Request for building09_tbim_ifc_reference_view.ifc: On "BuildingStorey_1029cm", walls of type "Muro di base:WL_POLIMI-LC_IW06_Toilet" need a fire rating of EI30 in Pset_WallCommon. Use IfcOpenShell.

First a look at what the model holds.

```python
import ifcopenshell
import ifcopenshell.util.element

model = ifcopenshell.open("building09_tbim_ifc_reference_view.ifc")
print(model.schema)
storey = next(s for s in model.by_type("IfcBuildingStorey") if s.Name == "BuildingStorey_1029cm")
walls = [e for e in ifcopenshell.util.element.get_decomposition(storey) if e.is_a("IfcWall")]
seen = {}
for e in walls:
    element_type = ifcopenshell.util.element.get_type(e)
    key = (element_type.Name if element_type != e and element_type else None, ifcopenshell.util.element.get_pset(e, "Pset_WallCommon", "FireRating"))
    seen[key] = seen.get(key, 0) + 1
for (name, value), count in sorted(seen.items(), key=str):
    print(count, "x", name, "|", value)
```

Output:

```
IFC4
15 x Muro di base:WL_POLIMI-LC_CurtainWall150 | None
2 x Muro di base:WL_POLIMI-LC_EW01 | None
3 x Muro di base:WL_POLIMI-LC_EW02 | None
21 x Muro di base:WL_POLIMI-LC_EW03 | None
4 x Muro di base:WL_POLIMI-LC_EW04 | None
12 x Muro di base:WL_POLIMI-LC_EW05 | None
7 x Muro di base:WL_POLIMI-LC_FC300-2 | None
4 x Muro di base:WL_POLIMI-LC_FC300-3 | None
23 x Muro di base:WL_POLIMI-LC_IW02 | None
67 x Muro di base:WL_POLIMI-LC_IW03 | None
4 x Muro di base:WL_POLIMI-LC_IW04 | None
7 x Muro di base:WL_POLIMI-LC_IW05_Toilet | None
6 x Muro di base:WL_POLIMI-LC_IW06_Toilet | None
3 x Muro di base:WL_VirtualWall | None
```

```python
import ifcopenshell
import ifcopenshell.api.pset
import ifcopenshell.util.element

model = ifcopenshell.open("building09_tbim_ifc_reference_view.ifc")

storey = next(s for s in model.by_type("IfcBuildingStorey") if s.Name == "BuildingStorey_1029cm")
walls = [e for e in ifcopenshell.util.element.get_decomposition(storey) if e.is_a("IfcWall")]

count = 0
for e in walls:
    element_type = ifcopenshell.util.element.get_type(e)
    if element_type in (None, e) or element_type.Name != "Muro di base:WL_POLIMI-LC_IW06_Toilet":
        continue
    # add_pset returns the element's existing set when there is one.
    pset = ifcopenshell.api.pset.add_pset(model, product=e, name="Pset_WallCommon")
    ifcopenshell.api.pset.edit_pset(model, pset=pset, properties={"FireRating": "EI30"})
    count += 1

print(count, "walls updated")

model.write("building09_tbim_ifc_reference_view_v2.ifc")
```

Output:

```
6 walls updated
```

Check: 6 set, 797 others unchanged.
